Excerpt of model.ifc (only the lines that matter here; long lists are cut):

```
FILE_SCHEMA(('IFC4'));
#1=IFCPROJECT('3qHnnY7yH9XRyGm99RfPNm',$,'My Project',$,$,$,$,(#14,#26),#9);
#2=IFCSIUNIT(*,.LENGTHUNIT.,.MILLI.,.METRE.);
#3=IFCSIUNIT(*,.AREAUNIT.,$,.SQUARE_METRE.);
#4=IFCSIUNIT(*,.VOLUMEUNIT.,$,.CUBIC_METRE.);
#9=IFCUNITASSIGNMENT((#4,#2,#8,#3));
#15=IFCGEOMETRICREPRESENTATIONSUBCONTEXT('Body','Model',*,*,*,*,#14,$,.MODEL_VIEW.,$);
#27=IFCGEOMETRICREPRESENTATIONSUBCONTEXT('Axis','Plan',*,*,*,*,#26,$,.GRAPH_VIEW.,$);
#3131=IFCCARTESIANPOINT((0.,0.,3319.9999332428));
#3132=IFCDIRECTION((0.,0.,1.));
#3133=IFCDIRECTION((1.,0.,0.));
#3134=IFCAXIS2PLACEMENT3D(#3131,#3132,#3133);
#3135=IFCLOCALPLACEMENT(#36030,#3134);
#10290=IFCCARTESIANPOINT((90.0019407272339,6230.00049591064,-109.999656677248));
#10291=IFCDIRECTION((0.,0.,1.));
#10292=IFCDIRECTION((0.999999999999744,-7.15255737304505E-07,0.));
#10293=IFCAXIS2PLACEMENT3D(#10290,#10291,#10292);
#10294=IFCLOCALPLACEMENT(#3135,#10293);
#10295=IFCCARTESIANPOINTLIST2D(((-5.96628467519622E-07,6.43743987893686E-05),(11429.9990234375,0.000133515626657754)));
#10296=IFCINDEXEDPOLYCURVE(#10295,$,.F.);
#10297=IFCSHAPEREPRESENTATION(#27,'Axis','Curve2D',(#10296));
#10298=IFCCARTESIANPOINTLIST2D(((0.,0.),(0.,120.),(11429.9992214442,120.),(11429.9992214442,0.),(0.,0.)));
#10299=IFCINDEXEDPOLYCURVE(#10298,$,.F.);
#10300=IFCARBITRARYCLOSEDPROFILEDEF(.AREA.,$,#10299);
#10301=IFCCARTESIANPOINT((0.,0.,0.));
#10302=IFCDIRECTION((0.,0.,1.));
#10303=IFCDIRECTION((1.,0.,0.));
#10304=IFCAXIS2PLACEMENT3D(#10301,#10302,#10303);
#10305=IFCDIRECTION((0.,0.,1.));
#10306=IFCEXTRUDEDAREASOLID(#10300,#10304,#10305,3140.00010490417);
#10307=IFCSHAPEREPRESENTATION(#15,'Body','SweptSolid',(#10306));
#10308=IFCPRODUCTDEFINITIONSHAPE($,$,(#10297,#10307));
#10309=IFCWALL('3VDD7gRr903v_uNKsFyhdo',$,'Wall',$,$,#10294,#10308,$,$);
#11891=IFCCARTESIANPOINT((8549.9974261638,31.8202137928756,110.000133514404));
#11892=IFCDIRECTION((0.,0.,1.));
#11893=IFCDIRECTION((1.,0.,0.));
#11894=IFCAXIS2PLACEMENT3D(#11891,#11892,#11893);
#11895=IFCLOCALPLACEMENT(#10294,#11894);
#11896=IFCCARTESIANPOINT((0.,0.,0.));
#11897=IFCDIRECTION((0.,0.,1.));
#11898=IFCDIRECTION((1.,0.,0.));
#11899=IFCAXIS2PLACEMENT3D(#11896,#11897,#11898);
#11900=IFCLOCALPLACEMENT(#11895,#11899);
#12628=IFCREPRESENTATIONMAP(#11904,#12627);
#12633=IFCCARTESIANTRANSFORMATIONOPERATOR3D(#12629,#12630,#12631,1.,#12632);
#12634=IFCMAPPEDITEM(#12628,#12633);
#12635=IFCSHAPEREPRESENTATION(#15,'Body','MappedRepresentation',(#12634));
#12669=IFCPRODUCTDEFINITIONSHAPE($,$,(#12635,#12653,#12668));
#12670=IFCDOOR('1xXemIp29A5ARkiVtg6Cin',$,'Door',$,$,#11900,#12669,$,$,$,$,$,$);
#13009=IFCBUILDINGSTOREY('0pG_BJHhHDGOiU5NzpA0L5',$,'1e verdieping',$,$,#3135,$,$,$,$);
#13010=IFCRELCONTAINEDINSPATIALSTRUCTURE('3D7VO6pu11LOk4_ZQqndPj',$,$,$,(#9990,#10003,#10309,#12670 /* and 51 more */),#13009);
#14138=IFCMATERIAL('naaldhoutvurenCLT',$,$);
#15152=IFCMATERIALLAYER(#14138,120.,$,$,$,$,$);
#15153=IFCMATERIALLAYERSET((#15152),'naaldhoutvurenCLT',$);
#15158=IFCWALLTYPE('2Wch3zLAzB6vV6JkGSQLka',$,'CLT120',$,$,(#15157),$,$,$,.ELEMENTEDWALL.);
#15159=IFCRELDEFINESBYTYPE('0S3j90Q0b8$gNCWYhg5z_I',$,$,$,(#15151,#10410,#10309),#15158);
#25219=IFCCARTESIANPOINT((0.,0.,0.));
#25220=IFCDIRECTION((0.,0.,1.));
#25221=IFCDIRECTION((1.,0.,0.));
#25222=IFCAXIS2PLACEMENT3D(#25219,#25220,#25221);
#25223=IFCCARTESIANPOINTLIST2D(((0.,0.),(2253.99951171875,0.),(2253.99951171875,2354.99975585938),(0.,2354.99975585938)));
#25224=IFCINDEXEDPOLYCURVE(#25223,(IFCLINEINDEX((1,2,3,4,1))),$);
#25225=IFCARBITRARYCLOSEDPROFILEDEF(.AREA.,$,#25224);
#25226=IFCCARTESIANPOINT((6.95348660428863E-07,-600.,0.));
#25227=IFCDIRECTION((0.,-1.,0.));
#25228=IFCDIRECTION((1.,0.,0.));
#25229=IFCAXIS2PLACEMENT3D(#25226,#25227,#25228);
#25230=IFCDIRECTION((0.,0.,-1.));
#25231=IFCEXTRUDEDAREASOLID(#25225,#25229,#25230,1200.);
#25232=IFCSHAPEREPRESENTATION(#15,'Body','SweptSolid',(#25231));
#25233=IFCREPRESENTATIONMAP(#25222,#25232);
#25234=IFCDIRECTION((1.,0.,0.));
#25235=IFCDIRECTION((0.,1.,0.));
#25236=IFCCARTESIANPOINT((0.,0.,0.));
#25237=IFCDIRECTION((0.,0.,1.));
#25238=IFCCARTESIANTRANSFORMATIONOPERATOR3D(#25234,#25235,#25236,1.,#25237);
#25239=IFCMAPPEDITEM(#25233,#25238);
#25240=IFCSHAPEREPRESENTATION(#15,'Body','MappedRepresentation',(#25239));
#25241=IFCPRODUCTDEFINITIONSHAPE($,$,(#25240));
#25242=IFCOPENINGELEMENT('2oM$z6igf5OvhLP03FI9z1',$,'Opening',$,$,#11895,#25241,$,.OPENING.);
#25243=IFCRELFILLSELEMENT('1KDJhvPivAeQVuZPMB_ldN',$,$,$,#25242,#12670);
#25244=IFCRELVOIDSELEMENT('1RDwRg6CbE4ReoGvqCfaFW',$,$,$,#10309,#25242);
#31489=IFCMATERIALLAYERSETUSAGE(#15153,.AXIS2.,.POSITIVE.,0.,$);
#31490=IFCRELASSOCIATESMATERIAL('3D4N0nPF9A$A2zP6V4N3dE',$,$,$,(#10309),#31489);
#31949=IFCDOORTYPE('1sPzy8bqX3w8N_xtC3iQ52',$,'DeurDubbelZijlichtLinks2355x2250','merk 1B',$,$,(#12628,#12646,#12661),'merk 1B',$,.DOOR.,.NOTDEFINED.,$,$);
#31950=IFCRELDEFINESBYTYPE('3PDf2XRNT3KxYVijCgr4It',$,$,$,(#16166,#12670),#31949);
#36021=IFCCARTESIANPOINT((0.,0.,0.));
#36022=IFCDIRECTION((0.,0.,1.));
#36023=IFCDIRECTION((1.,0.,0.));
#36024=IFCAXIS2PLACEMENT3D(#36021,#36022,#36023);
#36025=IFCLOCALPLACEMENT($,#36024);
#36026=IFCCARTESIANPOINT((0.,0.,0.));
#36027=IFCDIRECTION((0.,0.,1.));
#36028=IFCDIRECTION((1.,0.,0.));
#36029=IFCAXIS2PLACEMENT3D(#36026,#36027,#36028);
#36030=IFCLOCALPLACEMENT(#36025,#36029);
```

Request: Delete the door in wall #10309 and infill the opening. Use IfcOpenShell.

```python
import ifcopenshell
import ifcopenshell.api.feature
import ifcopenshell.api.root
import ifcopenshell.geom
import ifcopenshell.util.shape

model = ifcopenshell.open("model.ifc")
settings = ifcopenshell.geom.settings()


def volume(element):
    """Net volume in cubic metres, openings subtracted."""
    shape = ifcopenshell.geom.create_shape(settings, element)
    return ifcopenshell.util.shape.get_volume(shape.geometry)


door = model.by_guid("1xXemIp29A5ARkiVtg6Cin")
opening = door.FillsVoids[0].RelatingOpeningElement
wall = opening.VoidsElements[0].RelatingBuildingElement
before = volume(wall)

ifcopenshell.api.root.remove_product(model, product=door)
ifcopenshell.api.feature.remove_feature(model, feature=opening)

after = volume(wall)

print(f"wall volume {before:.3f} -> {after:.3f} m3")

model.write("model-out.ifc")
```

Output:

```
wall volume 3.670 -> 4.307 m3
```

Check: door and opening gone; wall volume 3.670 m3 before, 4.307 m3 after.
